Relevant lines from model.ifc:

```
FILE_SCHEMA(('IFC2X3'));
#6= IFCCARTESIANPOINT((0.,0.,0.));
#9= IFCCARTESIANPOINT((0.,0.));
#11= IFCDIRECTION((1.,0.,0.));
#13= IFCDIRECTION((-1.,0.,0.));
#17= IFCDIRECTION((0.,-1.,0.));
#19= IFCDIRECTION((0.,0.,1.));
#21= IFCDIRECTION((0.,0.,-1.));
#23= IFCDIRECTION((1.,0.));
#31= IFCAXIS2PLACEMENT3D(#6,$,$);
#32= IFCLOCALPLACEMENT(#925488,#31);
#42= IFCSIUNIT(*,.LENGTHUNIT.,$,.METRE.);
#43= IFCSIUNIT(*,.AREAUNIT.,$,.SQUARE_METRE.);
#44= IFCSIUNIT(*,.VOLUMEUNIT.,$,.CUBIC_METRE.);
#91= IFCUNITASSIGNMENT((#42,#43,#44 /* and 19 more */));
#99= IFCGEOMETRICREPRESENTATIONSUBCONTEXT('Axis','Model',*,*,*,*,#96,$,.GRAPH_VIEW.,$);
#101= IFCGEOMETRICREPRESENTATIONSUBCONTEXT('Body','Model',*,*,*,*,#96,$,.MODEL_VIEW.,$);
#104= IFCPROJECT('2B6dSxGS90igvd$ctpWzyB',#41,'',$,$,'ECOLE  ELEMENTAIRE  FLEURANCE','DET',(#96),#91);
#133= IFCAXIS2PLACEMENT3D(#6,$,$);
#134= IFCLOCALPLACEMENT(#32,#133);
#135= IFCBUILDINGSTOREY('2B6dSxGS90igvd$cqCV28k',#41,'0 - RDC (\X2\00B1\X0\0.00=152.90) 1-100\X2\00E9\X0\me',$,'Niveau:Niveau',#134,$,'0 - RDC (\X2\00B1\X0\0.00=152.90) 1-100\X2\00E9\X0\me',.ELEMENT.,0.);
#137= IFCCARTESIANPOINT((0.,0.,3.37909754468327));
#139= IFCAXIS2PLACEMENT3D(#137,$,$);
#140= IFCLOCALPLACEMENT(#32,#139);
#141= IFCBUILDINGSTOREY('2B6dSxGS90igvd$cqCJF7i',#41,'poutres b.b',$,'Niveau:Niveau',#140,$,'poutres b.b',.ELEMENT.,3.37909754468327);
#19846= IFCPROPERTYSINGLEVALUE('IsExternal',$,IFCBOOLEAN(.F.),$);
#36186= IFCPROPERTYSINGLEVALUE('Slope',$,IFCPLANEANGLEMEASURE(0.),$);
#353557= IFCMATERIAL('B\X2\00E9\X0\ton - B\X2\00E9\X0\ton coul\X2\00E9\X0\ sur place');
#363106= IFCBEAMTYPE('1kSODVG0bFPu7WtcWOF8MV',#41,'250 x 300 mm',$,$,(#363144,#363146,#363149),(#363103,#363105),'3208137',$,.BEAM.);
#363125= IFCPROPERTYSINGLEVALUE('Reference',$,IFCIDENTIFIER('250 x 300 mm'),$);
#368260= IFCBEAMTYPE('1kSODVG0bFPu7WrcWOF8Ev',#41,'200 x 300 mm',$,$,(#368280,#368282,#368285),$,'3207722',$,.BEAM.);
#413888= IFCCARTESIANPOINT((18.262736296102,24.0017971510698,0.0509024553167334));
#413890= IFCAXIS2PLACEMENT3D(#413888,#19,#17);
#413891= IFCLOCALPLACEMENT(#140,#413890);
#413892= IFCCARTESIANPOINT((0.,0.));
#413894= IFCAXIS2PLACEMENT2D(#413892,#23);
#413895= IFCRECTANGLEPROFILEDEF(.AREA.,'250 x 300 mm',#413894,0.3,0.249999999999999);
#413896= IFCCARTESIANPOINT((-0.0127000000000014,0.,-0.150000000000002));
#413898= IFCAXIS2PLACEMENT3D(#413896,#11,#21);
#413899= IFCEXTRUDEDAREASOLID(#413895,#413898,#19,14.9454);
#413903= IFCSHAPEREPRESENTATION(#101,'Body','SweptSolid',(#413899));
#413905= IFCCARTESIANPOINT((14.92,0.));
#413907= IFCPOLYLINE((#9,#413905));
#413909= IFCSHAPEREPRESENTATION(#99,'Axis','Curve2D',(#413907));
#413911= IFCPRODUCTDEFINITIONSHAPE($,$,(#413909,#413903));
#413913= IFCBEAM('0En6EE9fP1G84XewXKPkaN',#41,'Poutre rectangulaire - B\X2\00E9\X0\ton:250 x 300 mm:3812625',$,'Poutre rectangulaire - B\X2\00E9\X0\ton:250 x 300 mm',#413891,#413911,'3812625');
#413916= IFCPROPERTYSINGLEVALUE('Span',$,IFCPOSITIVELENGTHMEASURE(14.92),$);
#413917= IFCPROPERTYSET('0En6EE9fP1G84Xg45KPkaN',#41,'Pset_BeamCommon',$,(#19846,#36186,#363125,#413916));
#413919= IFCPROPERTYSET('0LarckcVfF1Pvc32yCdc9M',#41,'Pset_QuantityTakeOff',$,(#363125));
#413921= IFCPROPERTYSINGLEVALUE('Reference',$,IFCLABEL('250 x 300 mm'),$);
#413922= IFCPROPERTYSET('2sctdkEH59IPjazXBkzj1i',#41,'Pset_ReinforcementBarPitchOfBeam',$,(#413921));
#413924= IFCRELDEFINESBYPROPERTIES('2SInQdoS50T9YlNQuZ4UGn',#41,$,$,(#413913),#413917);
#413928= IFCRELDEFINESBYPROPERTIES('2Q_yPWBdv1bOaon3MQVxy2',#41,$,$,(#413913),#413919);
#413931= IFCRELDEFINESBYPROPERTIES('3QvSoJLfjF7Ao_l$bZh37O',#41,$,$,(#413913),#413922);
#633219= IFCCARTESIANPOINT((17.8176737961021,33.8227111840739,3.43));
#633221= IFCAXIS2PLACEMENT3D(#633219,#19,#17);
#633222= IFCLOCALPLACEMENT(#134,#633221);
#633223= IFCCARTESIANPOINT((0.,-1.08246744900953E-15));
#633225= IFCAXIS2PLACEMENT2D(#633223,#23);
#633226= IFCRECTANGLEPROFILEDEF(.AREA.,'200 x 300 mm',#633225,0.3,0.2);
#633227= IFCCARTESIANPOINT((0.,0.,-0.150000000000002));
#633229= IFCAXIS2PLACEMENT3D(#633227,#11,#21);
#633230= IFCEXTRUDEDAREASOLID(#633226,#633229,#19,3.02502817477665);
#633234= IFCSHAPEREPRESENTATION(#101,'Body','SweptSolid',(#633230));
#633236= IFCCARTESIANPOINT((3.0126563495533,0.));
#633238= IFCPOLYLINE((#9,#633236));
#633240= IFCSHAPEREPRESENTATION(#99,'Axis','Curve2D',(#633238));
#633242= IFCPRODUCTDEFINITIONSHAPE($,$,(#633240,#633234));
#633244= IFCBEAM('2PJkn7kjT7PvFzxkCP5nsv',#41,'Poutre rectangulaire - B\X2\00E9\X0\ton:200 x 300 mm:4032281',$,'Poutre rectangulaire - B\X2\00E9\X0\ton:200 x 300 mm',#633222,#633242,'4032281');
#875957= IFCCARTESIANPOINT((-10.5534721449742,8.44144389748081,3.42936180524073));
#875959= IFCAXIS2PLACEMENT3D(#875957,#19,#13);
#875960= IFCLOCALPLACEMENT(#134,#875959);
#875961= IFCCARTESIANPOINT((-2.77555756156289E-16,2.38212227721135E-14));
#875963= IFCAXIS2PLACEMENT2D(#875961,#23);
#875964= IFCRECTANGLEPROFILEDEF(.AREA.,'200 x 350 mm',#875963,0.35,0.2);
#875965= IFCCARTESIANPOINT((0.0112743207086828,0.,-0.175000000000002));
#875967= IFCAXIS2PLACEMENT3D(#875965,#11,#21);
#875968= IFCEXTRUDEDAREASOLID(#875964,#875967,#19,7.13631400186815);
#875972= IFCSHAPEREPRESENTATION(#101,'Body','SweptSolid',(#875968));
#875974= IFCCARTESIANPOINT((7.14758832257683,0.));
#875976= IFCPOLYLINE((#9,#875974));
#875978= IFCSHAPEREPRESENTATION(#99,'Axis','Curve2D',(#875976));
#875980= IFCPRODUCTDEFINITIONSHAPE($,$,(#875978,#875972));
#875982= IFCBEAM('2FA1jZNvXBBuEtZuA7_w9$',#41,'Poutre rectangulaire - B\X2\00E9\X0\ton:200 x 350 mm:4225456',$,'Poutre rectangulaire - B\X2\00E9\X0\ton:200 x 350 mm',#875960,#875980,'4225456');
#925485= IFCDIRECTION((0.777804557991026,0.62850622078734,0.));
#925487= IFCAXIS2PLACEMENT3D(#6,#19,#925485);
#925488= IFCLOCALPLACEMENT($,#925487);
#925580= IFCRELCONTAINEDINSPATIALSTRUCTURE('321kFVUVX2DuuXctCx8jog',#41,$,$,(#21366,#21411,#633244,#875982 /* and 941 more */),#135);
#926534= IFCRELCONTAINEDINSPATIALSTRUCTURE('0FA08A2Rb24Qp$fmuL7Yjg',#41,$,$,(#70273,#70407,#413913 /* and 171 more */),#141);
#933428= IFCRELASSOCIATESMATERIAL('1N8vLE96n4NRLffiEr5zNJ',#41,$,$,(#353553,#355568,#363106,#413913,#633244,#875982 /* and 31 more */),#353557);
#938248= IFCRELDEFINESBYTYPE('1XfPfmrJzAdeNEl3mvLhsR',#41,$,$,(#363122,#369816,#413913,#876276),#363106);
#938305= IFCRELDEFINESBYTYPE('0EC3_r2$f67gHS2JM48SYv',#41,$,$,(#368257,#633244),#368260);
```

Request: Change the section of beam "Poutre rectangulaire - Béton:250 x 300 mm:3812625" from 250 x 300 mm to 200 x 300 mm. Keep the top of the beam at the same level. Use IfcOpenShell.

```python
import ifcopenshell
import ifcopenshell.api.pset
import ifcopenshell.api.type
import ifcopenshell.util.element
import ifcopenshell.util.representation

model = ifcopenshell.open("model.ifc")

member = model.by_guid("0En6EE9fP1G84XewXKPkaN")
source = next(p for p in model.by_type("IfcRectangleProfileDef") if p.ProfileName == "200 x 300 mm")

body = ifcopenshell.util.representation.get_representation(member, "Model", "Body")
solid = body.Items[0]
old_profile = solid.SweptArea

# Copy the section's sizes but keep this member's own profile position.
profile = ifcopenshell.util.element.copy(model, source)
# Profiles are centred, so shift by half the change in depth to hold the top.
shift = (old_profile.XDim - profile.XDim) / 2
x, y = old_profile.Position.Location.Coordinates
up = (-1.0, 0.0)  # upwards, in the solid's own plane
location = model.createIfcCartesianPoint((x + up[0] * shift, y + up[1] * shift))
profile.Position = model.createIfcAxis2Placement2D(location, old_profile.Position.RefDirection)
solid.SweptArea = profile
if not model.get_total_inverses(old_profile):
    ifcopenshell.util.element.remove_deep2(model, old_profile)

new_type = model.by_guid("1kSODVG0bFPu7WrcWOF8Ev")
ifcopenshell.api.type.assign_type(
    model, related_objects=[member], relating_type=new_type, should_map_representations=False
)
member.Name = member.Name.replace("250 x 300 mm", "200 x 300 mm")
member.ObjectType = "Poutre rectangulaire - Béton:200 x 300 mm"
pset = model.by_id(ifcopenshell.util.element.get_pset(member, "Pset_BeamCommon", should_inherit=False)["id"])
ifcopenshell.api.pset.edit_pset(model, pset=pset, properties={"Reference": "200 x 300 mm"})
pset = model.by_id(ifcopenshell.util.element.get_pset(member, "Pset_QuantityTakeOff", should_inherit=False)["id"])
ifcopenshell.api.pset.edit_pset(model, pset=pset, properties={"Reference": "200 x 300 mm"})
pset = model.by_id(ifcopenshell.util.element.get_pset(member, "Pset_ReinforcementBarPitchOfBeam", should_inherit=False)["id"])
ifcopenshell.api.pset.edit_pset(model, pset=pset, properties={"Reference": "200 x 300 mm"})

print(solid.SweptArea)

model.write("model_updated.ifc")
```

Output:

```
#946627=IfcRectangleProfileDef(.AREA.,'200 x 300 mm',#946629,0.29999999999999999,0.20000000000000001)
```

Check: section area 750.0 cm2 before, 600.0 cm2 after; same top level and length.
